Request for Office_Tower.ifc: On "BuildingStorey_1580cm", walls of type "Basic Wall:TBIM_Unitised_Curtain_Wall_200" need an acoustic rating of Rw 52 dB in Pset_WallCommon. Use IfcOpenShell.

First a look at what the model holds.

```python
import ifcopenshell
import ifcopenshell.util.element

model = ifcopenshell.open("Office_Tower.ifc")
print(model.schema)
storey = next(s for s in model.by_type("IfcBuildingStorey") if s.Name == "BuildingStorey_1580cm")
walls = [e for e in ifcopenshell.util.element.get_decomposition(storey) if e.is_a("IfcWall")]
seen = {}
for e in walls:
    element_type = ifcopenshell.util.element.get_type(e)
    key = (element_type.Name if element_type != e and element_type else None, ifcopenshell.util.element.get_pset(e, "Pset_WallCommon", "AcousticRating"))
    seen[key] = seen.get(key, 0) + 1
for (name, value), count in sorted(seen.items(), key=str):
    print(count, "x", name, "|", value)
```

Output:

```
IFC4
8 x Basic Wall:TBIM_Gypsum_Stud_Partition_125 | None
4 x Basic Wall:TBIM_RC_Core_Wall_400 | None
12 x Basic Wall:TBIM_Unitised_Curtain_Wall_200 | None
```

```python
import ifcopenshell
import ifcopenshell.api.pset
import ifcopenshell.util.element

model = ifcopenshell.open("Office_Tower.ifc")

storey = next(s for s in model.by_type("IfcBuildingStorey") if s.Name == "BuildingStorey_1580cm")
walls = [e for e in ifcopenshell.util.element.get_decomposition(storey) if e.is_a("IfcWall")]

count = 0
for e in walls:
    element_type = ifcopenshell.util.element.get_type(e)
    if element_type in (None, e) or element_type.Name != "Basic Wall:TBIM_Unitised_Curtain_Wall_200":
        continue
    # add_pset returns the element's existing set when there is one.
    pset = ifcopenshell.api.pset.add_pset(model, product=e, name="Pset_WallCommon")
    ifcopenshell.api.pset.edit_pset(model, pset=pset, properties={"AcousticRating": "Rw 52 dB"})
    count += 1

print(count, "walls updated")

model.write("Office_Tower_v2.ifc")
```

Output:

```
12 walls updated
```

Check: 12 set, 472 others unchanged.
